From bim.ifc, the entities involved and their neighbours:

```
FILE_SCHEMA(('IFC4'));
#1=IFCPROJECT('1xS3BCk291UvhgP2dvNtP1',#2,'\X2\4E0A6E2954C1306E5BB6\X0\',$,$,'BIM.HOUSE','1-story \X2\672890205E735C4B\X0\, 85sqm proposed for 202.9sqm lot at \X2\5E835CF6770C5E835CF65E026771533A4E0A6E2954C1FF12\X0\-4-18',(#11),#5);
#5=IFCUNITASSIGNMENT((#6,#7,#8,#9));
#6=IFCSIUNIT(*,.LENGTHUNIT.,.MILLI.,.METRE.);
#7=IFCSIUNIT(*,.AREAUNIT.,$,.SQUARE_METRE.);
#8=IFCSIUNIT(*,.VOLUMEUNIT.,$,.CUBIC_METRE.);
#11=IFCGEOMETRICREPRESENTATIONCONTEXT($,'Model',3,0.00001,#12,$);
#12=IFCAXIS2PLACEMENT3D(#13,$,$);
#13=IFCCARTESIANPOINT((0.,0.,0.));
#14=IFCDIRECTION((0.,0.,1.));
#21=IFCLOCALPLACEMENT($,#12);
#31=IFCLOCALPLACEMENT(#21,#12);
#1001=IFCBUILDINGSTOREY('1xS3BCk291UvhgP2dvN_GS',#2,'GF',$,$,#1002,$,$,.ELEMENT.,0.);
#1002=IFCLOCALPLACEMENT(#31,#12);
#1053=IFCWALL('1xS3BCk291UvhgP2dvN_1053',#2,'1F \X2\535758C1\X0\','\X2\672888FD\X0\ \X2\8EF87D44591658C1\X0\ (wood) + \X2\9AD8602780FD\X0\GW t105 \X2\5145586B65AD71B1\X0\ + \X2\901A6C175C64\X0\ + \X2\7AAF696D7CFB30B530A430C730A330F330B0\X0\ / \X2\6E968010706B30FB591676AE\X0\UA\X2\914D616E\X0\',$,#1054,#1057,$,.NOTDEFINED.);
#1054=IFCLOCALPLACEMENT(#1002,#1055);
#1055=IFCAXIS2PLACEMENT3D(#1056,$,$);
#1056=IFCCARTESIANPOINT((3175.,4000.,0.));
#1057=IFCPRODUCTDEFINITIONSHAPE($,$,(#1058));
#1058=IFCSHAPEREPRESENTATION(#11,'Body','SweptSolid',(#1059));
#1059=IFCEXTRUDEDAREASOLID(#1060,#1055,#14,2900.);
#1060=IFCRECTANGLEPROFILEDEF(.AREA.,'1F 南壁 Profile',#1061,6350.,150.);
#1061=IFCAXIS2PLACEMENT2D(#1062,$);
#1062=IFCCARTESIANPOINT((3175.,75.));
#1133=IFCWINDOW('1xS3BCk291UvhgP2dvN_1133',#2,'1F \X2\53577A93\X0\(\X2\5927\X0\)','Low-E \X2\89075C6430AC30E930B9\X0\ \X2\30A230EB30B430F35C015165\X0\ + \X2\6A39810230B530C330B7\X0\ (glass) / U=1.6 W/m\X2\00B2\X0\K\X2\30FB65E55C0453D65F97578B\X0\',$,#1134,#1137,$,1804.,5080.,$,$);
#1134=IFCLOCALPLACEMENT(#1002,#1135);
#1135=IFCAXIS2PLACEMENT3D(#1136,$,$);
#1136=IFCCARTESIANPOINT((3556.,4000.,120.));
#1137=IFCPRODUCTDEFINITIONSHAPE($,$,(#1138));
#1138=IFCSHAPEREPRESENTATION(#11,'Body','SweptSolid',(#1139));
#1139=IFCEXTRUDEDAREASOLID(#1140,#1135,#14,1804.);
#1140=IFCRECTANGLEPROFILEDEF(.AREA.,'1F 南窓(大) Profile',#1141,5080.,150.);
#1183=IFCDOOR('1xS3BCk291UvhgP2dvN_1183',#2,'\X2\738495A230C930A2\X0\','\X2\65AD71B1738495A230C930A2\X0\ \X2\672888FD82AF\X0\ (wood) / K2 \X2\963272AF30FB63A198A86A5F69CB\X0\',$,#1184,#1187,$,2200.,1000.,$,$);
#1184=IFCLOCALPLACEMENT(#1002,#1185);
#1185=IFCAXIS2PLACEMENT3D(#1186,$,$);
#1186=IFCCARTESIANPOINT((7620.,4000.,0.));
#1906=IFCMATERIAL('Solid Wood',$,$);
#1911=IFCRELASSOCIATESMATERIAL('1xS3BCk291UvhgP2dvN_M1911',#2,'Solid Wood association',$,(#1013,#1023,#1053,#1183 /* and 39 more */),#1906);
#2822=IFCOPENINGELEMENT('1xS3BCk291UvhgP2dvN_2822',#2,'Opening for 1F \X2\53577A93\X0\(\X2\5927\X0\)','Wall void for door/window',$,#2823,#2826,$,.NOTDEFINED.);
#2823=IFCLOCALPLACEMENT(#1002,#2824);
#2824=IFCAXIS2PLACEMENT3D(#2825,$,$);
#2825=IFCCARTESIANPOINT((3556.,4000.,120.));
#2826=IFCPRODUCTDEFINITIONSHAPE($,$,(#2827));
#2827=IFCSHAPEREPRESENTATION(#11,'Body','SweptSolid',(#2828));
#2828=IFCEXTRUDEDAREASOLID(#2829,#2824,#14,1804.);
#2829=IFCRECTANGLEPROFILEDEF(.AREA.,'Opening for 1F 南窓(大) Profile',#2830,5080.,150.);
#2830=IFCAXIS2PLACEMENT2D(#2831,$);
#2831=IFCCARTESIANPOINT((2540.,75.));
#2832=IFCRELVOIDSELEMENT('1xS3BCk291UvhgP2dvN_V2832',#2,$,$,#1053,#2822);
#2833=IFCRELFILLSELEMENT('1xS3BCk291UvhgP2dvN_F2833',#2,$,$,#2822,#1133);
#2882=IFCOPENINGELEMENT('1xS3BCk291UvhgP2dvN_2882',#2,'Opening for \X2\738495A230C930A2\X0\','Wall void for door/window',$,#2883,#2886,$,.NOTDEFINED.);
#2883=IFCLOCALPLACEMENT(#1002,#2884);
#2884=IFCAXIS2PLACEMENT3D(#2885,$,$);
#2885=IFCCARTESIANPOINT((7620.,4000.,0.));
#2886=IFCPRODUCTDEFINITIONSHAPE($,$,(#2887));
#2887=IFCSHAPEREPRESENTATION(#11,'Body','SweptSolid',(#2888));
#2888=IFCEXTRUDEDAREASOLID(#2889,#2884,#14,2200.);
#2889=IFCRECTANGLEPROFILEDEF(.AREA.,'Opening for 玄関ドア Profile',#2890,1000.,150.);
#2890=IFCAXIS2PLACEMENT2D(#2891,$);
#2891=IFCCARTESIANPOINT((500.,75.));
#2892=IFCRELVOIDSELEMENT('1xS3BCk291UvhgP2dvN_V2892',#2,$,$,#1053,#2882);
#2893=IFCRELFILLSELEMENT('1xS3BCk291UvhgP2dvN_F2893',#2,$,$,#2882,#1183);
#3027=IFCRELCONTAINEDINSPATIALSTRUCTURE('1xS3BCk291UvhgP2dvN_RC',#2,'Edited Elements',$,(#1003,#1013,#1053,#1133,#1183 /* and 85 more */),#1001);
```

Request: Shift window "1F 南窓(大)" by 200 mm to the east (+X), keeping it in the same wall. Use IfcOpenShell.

```python
import ifcopenshell
import ifcopenshell.api.geometry
import ifcopenshell.util.placement

model = ifcopenshell.open("bim.ifc")

window = model.by_guid("1xS3BCk291UvhgP2dvN_1133")
opening = window.FillsVoids[0].RelatingOpeningElement
wall = opening.VoidsElements[0].RelatingBuildingElement

wall_matrix = ifcopenshell.util.placement.get_local_placement(wall.ObjectPlacement)
shift = wall_matrix[:3, 0] * 200.0
before = ifcopenshell.util.placement.get_local_placement(window.ObjectPlacement)[:3, 3].copy()

# The window is not placed relative to its opening, so move both.
for product in (opening, window):
    matrix = ifcopenshell.util.placement.get_local_placement(product.ObjectPlacement)
    matrix[:3, 3] += shift
    ifcopenshell.api.geometry.edit_object_placement(model, product=product, matrix=matrix, is_si=False)

after = ifcopenshell.util.placement.get_local_placement(window.ObjectPlacement)[:3, 3]
print("window moved by", (after - before).round(3) + 0.0)

model.write("bim_rev.ifc")
```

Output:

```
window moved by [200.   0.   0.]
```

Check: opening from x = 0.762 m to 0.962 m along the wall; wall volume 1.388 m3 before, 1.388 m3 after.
